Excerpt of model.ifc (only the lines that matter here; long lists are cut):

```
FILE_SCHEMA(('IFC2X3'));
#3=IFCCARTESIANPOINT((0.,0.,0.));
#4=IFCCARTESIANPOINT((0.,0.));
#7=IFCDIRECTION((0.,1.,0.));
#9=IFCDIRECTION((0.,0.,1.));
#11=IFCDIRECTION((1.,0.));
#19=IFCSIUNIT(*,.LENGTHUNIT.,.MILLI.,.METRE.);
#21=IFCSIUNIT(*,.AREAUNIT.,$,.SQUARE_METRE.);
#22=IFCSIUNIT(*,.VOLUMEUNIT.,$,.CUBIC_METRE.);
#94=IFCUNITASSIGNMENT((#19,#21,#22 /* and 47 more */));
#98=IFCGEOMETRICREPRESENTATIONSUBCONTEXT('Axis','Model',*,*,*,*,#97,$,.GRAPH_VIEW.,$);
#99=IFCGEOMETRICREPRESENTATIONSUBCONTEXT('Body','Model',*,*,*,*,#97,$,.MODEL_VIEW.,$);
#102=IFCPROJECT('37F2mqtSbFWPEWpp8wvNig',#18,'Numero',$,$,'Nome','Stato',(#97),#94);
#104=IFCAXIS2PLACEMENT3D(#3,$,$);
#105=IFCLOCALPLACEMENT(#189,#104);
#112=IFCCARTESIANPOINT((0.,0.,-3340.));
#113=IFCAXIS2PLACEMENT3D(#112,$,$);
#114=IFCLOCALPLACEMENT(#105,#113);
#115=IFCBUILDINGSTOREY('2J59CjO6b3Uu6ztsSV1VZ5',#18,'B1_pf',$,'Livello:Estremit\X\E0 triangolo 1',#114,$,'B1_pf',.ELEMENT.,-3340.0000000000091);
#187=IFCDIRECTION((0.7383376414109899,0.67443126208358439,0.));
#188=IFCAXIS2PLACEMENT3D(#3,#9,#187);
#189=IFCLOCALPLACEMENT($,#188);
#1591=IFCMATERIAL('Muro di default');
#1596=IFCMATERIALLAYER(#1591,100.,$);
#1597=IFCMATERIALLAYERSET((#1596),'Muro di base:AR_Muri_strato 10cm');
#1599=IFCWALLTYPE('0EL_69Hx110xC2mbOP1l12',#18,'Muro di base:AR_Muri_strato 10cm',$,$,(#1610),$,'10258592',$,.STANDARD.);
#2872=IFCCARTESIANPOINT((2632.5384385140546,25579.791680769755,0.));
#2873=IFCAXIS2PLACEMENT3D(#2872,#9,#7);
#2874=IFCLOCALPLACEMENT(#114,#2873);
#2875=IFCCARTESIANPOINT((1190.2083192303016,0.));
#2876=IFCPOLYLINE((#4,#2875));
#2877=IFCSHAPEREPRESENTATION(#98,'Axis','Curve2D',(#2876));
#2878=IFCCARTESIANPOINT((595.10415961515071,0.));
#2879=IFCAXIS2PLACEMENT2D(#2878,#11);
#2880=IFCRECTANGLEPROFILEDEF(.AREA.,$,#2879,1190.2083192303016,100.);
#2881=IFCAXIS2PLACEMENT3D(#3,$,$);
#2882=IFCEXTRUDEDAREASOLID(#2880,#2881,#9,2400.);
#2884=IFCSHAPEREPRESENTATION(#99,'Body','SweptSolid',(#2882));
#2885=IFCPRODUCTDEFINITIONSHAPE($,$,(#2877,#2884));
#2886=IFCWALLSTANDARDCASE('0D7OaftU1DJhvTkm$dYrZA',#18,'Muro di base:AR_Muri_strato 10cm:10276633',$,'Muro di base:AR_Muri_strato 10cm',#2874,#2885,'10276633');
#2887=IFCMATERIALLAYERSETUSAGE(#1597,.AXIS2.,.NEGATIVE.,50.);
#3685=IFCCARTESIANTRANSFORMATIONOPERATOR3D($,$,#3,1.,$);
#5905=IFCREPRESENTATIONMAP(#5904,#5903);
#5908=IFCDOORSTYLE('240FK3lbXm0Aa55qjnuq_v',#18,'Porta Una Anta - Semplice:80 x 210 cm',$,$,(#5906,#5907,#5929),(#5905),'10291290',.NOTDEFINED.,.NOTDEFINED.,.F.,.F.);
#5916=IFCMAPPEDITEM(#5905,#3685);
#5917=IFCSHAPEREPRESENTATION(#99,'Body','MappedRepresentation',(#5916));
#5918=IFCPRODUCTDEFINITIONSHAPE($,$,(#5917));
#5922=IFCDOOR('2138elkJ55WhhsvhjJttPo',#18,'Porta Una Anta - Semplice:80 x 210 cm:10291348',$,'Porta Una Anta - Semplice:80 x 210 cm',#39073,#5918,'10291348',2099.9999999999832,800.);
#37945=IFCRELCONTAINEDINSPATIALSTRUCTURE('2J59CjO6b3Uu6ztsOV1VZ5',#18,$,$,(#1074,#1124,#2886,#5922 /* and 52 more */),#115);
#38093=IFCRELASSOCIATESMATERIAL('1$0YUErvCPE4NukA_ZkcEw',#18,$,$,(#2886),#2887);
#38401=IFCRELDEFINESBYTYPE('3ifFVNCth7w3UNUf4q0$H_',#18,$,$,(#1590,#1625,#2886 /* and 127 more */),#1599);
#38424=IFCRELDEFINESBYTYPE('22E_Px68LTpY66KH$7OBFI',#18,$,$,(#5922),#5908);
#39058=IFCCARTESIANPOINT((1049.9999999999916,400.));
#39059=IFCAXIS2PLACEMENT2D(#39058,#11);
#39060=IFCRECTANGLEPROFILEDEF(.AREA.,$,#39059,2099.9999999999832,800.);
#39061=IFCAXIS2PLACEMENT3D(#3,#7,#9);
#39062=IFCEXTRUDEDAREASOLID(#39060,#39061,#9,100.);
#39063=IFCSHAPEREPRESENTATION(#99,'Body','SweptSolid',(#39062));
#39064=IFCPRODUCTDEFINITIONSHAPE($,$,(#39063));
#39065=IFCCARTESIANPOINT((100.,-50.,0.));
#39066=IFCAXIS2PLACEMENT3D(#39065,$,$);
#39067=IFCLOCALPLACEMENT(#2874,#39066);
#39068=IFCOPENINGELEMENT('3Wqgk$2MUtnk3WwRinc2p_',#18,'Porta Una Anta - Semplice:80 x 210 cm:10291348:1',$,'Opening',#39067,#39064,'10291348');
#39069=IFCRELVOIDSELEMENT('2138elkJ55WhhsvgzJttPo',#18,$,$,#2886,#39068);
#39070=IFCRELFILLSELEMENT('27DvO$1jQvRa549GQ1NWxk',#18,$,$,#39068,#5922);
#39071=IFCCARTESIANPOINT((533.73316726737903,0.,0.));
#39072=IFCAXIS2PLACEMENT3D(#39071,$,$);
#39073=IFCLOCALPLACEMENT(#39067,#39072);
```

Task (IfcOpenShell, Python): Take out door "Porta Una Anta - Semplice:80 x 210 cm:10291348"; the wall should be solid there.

```python
import ifcopenshell
import ifcopenshell.api.feature
import ifcopenshell.api.root
import ifcopenshell.geom
import ifcopenshell.util.shape

model = ifcopenshell.open("model.ifc")
settings = ifcopenshell.geom.settings()


def volume(element):
    """Net volume in cubic metres, openings subtracted."""
    shape = ifcopenshell.geom.create_shape(settings, element)
    return ifcopenshell.util.shape.get_volume(shape.geometry)


door = model.by_guid("2138elkJ55WhhsvhjJttPo")
opening = door.FillsVoids[0].RelatingOpeningElement
wall = opening.VoidsElements[0].RelatingBuildingElement
before = volume(wall)

ifcopenshell.api.root.remove_product(model, product=door)
ifcopenshell.api.feature.remove_feature(model, feature=opening)

after = volume(wall)

print(f"wall volume {before:.3f} -> {after:.3f} m3")

model.write("model-out.ifc")
```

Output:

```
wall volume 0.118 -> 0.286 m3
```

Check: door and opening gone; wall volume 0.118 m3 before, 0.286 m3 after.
